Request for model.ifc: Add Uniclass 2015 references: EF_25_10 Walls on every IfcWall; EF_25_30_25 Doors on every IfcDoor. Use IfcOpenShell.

First a look at what the model holds.

```python
import ifcopenshell

model = ifcopenshell.open("model.ifc")
print(model.schema)
print("classifications:", [c.Name for c in model.by_type("IfcClassification")])
for ifc_class in ("IfcDoor", "IfcRoof", "IfcStair", "IfcWall", "IfcWindow"):
    print(ifc_class, len(model.by_type(ifc_class)))
```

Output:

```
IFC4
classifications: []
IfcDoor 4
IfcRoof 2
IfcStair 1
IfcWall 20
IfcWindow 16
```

```python
import ifcopenshell
import ifcopenshell.api.classification

model = ifcopenshell.open("model.ifc")

system = ifcopenshell.api.classification.add_classification(model, classification="Uniclass 2015")

codes = {
    "IfcWall": ("EF_25_10", "Walls"),
    "IfcDoor": ("EF_25_30_25", "Doors"),
}
for ifc_class, (code, name) in codes.items():
    products = model.by_type(ifc_class)
    ifcopenshell.api.classification.add_reference(
        model, products=products, classification=system, identification=code, name=name
    )
    print(code, len(products))

model.write("model_updated.ifc")
```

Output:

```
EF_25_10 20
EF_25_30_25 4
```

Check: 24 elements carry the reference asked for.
